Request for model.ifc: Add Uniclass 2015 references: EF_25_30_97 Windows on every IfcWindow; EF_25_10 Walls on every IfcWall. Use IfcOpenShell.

First a look at what the model holds.

```python
import ifcopenshell

model = ifcopenshell.open("model.ifc")
print(model.schema)
print("classifications:", [c.Name for c in model.by_type("IfcClassification")])
for ifc_class in ("IfcDoor", "IfcRoof", "IfcStair", "IfcWall", "IfcWindow"):
    print(ifc_class, len(model.by_type(ifc_class)))
```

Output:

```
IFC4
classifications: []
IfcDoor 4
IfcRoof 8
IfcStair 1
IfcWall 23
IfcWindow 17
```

```python
import ifcopenshell
import ifcopenshell.api.classification

model = ifcopenshell.open("model.ifc")

system = ifcopenshell.api.classification.add_classification(model, classification="Uniclass 2015")

codes = {
    "IfcWindow": ("EF_25_30_97", "Windows"),
    "IfcWall": ("EF_25_10", "Walls"),
}
for ifc_class, (code, name) in codes.items():
    products = model.by_type(ifc_class)
    ifcopenshell.api.classification.add_reference(
        model, products=products, classification=system, identification=code, name=name
    )
    print(code, len(products))

model.write("model_rev.ifc")
```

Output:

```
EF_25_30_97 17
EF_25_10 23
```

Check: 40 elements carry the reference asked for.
